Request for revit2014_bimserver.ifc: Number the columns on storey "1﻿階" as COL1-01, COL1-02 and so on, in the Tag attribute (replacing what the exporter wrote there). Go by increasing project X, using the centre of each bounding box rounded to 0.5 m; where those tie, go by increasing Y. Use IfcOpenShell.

First a look at what the model holds.

```python
import ifcopenshell
import ifcopenshell.util.element
import ifcopenshell.util.placement

model = ifcopenshell.open("revit2014_bimserver.ifc")
print(model.schema)
storey = next(s for s in model.by_type("IfcBuildingStorey") if s.Name == '1\ufeff階')
columns = [e for e in ifcopenshell.util.element.get_decomposition(storey) if e.is_a("IfcColumn")]
for e in sorted(columns, key=lambda e: e.id()):
    origin = ifcopenshell.util.placement.get_local_placement(e.ObjectPlacement)[:3, 3]
    print(e.id(), e.Tag, e.Name, origin.round(2) + 0.0, sep=" | ")
```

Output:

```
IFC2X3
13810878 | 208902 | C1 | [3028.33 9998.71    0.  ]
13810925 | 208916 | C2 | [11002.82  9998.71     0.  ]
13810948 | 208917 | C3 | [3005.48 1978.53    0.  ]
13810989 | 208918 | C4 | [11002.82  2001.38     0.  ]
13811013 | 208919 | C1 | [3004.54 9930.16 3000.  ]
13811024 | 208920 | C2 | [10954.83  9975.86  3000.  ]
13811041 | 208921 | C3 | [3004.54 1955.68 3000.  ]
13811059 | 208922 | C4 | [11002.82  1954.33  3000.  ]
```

```python
import ifcopenshell
import ifcopenshell.geom
import ifcopenshell.util.element
import ifcopenshell.util.shape

model = ifcopenshell.open("revit2014_bimserver.ifc")
settings = ifcopenshell.geom.settings()
settings.set("use-world-coords", True)


def centre(element):
    shape = ifcopenshell.geom.create_shape(settings, element)
    return ifcopenshell.util.shape.get_bbox_centroid(shape.geometry)


storey = next(s for s in model.by_type("IfcBuildingStorey") if s.Name == '1\ufeff階')
columns = [e for e in ifcopenshell.util.element.get_decomposition(storey) if e.is_a("IfcColumn")]

# Insertion points can sit at a corner or the storey origin, so sort by the geometry (in metres).
centres = {e: centre(e) for e in columns}
columns.sort(key=lambda e: (round(centres[e][0] / 0.5), centres[e][1]))

for i, e in enumerate(columns, start=1):
    number = f"COL1-{i:02d}"
    e.Tag = number
    print(e.id(), number)

model.write("revit2014_bimserver-out.ifc")
```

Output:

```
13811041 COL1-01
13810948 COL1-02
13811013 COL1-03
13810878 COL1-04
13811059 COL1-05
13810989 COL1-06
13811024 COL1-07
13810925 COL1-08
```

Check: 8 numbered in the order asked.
